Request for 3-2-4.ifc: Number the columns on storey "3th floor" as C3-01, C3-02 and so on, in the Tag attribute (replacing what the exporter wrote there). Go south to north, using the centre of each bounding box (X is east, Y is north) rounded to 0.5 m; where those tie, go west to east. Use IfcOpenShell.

First a look at what the model holds.

```python
import ifcopenshell
import ifcopenshell.util.element
import ifcopenshell.util.placement

model = ifcopenshell.open("3-2-4.ifc")
print(model.schema)
storey = next(s for s in model.by_type("IfcBuildingStorey") if s.Name == "3th floor")
columns = [e for e in ifcopenshell.util.element.get_decomposition(storey) if e.is_a("IfcColumn")]
for e in sorted(columns, key=lambda e: e.id()):
    origin = ifcopenshell.util.placement.get_local_placement(e.ObjectPlacement)[:3, 3]
    print(e.id(), e.Tag, e.Name, origin.round(2) + 0.0, sep=" | ")
```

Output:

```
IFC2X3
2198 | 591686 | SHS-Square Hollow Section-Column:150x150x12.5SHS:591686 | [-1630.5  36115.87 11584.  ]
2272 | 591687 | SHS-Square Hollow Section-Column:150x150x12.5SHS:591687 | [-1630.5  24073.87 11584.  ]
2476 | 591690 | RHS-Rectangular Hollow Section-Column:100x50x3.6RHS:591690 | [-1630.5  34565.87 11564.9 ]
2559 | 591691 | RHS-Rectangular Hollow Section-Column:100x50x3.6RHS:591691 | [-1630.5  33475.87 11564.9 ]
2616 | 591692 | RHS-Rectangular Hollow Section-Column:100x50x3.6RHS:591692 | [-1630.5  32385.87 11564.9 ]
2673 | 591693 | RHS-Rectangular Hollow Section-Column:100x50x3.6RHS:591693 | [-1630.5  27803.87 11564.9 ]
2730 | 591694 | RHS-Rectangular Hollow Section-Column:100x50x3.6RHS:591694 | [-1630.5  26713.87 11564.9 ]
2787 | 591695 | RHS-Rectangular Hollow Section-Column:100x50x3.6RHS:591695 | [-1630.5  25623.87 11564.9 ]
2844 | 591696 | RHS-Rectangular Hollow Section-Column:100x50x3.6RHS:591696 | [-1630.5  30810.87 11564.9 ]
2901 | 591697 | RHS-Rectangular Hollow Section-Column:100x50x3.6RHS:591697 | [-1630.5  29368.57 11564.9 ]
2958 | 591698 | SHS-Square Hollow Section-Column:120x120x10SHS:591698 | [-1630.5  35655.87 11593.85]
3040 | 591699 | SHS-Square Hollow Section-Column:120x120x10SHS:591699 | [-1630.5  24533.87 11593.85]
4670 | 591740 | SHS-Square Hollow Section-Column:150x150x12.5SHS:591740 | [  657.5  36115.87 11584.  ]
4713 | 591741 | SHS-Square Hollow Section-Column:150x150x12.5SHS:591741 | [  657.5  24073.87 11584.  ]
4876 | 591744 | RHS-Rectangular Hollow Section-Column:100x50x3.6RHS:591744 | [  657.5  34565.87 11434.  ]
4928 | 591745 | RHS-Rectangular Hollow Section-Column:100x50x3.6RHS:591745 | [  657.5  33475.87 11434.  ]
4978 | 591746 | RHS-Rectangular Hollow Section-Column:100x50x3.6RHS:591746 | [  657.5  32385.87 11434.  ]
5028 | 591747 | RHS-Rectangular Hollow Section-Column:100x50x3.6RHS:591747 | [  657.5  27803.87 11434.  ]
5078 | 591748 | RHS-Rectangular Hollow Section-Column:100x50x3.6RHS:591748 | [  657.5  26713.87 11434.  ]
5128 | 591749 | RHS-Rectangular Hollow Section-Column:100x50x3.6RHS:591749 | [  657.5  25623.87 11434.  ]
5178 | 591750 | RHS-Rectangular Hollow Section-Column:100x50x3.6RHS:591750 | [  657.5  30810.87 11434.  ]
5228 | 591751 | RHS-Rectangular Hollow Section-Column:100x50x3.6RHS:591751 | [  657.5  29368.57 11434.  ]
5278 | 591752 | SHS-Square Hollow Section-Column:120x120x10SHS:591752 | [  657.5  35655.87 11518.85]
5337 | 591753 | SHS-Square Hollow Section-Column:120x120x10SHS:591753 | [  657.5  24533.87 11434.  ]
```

```python
import ifcopenshell
import ifcopenshell.geom
import ifcopenshell.util.element
import ifcopenshell.util.shape

model = ifcopenshell.open("3-2-4.ifc")
settings = ifcopenshell.geom.settings()
settings.set("use-world-coords", True)


def centre(element):
    shape = ifcopenshell.geom.create_shape(settings, element)
    return ifcopenshell.util.shape.get_bbox_centroid(shape.geometry)


storey = next(s for s in model.by_type("IfcBuildingStorey") if s.Name == "3th floor")
columns = [e for e in ifcopenshell.util.element.get_decomposition(storey) if e.is_a("IfcColumn")]

# Insertion points can sit at a corner or the storey origin, so sort by the geometry (in metres).
centres = {e: centre(e) for e in columns}
columns.sort(key=lambda e: (round(centres[e][1] / 0.5), centres[e][0]))

for i, e in enumerate(columns, start=1):
    number = f"C3-{i:02d}"
    e.Tag = number
    print(e.id(), number)

model.write("3-2-4_v2.ifc")
```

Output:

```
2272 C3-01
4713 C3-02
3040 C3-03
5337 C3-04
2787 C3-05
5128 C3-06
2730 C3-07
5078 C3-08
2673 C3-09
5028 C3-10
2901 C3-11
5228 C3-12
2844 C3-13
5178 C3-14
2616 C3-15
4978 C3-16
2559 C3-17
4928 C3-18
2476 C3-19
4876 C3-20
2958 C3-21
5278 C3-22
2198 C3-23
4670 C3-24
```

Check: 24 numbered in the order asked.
